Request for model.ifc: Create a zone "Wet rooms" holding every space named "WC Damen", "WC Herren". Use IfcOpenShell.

First a look at what the model holds.

```python
import ifcopenshell

model = ifcopenshell.open("model.ifc")
print(model.schema)
seen = {}
for space in model.by_type("IfcSpace"):
    seen[space.LongName] = seen.get(space.LongName, 0) + 1
for name, count in sorted(seen.items(), key=str):
    print(count, "x", name)
print("zones:", [z.Name for z in model.by_type("IfcZone")][:20])
```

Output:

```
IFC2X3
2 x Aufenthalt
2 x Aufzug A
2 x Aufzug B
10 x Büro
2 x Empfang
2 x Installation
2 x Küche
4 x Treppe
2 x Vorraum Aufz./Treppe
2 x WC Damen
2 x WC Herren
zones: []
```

```python
import ifcopenshell
import ifcopenshell.api.group
import ifcopenshell.api.root

model = ifcopenshell.open("model.ifc")

names = {"WC Damen", "WC Herren"}
spaces = [s for s in model.by_type("IfcSpace") if s.LongName in names]

zone = ifcopenshell.api.root.create_entity(model, ifc_class="IfcZone", name="Wet rooms")
ifcopenshell.api.group.assign_group(model, products=spaces, group=zone)
print(len(spaces), "spaces in", zone.Name)

model.write("model_rev.ifc")
```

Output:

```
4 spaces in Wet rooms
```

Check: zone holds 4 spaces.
